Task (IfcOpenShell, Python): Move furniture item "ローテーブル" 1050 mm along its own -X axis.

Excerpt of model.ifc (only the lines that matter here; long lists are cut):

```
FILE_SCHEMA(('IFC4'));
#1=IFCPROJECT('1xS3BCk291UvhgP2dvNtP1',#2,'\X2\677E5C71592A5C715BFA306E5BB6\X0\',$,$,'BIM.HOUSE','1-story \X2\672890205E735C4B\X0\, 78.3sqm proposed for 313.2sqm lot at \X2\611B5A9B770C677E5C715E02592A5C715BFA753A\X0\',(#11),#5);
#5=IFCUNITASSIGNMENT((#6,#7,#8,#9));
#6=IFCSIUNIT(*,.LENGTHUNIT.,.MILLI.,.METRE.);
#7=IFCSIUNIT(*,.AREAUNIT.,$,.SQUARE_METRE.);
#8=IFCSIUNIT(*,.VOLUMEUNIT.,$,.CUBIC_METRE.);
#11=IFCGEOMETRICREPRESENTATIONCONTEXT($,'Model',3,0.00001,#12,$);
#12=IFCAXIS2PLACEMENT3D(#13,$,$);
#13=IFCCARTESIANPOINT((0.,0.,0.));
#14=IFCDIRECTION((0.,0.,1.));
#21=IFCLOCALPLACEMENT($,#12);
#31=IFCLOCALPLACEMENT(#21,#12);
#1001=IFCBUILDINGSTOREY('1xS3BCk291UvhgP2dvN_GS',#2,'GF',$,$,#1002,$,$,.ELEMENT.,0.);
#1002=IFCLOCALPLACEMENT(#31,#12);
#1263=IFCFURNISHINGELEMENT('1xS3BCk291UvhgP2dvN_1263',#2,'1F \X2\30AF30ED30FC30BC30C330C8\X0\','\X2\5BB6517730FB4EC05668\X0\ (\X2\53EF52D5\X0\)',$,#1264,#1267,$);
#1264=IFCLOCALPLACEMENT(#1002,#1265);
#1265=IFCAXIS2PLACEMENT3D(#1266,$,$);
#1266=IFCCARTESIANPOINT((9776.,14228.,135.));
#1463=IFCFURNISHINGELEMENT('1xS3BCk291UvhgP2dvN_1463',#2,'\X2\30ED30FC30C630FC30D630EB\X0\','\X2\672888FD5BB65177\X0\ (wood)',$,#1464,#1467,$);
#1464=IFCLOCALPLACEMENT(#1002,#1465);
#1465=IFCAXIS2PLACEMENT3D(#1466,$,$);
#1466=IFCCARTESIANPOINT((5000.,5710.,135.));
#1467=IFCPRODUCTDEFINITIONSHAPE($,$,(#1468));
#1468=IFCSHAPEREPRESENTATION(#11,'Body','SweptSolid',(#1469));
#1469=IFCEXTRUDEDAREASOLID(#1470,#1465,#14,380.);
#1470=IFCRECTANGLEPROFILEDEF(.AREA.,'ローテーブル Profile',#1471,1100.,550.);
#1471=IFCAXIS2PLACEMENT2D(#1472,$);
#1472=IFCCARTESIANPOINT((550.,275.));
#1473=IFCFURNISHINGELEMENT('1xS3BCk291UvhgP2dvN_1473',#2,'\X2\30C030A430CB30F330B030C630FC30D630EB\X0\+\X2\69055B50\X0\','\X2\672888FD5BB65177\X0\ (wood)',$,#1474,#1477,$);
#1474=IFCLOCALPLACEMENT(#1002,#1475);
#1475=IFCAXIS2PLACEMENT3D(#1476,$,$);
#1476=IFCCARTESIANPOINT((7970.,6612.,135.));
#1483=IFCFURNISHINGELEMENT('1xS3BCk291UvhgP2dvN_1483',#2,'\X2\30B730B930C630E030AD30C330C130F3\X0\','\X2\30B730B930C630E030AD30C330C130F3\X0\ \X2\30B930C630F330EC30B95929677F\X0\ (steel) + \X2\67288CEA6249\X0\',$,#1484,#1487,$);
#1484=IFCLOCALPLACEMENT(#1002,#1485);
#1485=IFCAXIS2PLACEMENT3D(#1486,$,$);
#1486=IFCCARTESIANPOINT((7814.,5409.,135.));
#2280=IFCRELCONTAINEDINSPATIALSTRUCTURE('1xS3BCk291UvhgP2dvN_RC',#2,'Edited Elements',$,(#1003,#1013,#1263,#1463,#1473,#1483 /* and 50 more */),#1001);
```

```python
import ifcopenshell
import ifcopenshell.api.geometry
import ifcopenshell.util.placement

model = ifcopenshell.open("model.ifc")

item = model.by_guid("1xS3BCk291UvhgP2dvN_1463")
matrix = ifcopenshell.util.placement.get_local_placement(item.ObjectPlacement)
matrix[:3, 3] -= matrix[:3, 0] * 1050.0
ifcopenshell.api.geometry.edit_object_placement(model, product=item, matrix=matrix, is_si=False)

print(ifcopenshell.util.placement.get_local_placement(item.ObjectPlacement).round(3) + 0.0)

model.write("model_v2.ifc")
```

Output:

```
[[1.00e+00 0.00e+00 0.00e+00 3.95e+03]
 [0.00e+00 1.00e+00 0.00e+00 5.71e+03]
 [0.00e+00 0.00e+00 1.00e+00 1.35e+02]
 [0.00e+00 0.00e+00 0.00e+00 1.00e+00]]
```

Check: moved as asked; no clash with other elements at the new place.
